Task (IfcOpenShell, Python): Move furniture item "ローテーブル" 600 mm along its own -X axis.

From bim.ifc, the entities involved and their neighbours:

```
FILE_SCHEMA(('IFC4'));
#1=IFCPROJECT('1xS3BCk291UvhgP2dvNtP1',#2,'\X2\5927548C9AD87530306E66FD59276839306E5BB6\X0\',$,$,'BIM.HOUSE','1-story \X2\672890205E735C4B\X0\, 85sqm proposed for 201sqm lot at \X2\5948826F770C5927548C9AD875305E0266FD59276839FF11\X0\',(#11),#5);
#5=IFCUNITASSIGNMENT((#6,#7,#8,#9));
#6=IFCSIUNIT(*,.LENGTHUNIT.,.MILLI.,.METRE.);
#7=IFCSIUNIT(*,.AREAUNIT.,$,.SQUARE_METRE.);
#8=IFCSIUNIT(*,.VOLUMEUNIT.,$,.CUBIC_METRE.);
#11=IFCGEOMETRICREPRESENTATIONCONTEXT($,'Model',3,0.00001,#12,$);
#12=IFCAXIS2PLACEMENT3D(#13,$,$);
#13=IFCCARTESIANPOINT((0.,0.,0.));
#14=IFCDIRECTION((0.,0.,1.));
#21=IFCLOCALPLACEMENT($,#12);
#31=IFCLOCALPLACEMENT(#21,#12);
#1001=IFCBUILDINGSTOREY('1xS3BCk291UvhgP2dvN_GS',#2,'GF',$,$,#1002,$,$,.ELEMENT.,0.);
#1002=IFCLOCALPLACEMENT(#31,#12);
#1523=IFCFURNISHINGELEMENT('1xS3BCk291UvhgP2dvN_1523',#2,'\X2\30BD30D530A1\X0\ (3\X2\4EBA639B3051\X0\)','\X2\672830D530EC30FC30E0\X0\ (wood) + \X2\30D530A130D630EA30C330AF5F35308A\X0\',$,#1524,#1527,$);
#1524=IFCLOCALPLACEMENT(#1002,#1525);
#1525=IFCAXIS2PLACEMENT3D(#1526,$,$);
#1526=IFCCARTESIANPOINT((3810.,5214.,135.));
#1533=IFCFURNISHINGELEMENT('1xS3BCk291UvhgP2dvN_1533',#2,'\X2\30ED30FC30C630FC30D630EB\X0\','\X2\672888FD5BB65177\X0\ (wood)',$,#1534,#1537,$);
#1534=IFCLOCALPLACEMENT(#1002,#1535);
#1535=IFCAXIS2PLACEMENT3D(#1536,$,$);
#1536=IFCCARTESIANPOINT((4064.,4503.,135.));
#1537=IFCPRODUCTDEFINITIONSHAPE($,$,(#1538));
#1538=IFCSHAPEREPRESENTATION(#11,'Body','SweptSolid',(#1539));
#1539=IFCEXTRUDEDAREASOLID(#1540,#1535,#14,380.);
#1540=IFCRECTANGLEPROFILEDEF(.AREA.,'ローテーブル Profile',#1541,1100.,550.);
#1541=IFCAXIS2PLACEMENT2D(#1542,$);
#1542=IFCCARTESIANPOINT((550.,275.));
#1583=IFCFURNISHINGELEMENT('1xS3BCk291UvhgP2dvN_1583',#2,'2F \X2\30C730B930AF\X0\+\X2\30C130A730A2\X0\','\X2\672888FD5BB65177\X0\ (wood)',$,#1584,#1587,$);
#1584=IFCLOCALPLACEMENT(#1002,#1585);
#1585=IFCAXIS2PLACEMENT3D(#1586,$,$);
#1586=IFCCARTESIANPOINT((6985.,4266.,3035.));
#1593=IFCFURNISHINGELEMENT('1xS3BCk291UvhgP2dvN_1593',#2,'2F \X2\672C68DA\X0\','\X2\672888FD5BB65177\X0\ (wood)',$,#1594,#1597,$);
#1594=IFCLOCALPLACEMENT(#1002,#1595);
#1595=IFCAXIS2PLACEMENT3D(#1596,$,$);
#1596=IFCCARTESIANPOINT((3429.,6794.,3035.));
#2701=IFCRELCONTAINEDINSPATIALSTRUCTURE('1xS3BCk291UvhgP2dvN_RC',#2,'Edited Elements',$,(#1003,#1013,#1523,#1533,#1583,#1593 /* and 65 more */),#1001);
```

```python
import ifcopenshell
import ifcopenshell.api.geometry
import ifcopenshell.util.placement
import ifcopenshell.util.unit

model = ifcopenshell.open("bim.ifc")
unit_scale = ifcopenshell.util.unit.calculate_unit_scale(model)

item = model.by_guid("1xS3BCk291UvhgP2dvN_1533")
matrix = ifcopenshell.util.placement.get_local_placement(item.ObjectPlacement)
matrix[:3, 3] -= matrix[:3, 0] * 0.6 / unit_scale
ifcopenshell.api.geometry.edit_object_placement(model, product=item, matrix=matrix, is_si=False)

print(ifcopenshell.util.placement.get_local_placement(item.ObjectPlacement).round(3) + 0.0)

model.write("bim_edited.ifc")
```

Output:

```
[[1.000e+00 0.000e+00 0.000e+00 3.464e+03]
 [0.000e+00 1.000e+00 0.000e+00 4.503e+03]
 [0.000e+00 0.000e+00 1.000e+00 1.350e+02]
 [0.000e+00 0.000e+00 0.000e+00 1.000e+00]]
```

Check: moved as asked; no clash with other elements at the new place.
